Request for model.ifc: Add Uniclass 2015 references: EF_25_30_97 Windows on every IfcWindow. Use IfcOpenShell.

First a look at what the model holds.

```python
import ifcopenshell

model = ifcopenshell.open("model.ifc")
print(model.schema)
print("classifications:", [c.Name for c in model.by_type("IfcClassification")])
for ifc_class in ("IfcDoor", "IfcRoof", "IfcStair", "IfcWall", "IfcWindow"):
    print(ifc_class, len(model.by_type(ifc_class)))
```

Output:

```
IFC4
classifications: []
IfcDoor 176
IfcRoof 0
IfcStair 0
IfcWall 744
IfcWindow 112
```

```python
import ifcopenshell
import ifcopenshell.api.classification

model = ifcopenshell.open("model.ifc")

system = ifcopenshell.api.classification.add_classification(model, classification="Uniclass 2015")

codes = {
    "IfcWindow": ("EF_25_30_97", "Windows"),
}
for ifc_class, (code, name) in codes.items():
    products = model.by_type(ifc_class)
    ifcopenshell.api.classification.add_reference(
        model, products=products, classification=system, identification=code, name=name
    )
    print(code, len(products))

model.write("model_updated.ifc")
```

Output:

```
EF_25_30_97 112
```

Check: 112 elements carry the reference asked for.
